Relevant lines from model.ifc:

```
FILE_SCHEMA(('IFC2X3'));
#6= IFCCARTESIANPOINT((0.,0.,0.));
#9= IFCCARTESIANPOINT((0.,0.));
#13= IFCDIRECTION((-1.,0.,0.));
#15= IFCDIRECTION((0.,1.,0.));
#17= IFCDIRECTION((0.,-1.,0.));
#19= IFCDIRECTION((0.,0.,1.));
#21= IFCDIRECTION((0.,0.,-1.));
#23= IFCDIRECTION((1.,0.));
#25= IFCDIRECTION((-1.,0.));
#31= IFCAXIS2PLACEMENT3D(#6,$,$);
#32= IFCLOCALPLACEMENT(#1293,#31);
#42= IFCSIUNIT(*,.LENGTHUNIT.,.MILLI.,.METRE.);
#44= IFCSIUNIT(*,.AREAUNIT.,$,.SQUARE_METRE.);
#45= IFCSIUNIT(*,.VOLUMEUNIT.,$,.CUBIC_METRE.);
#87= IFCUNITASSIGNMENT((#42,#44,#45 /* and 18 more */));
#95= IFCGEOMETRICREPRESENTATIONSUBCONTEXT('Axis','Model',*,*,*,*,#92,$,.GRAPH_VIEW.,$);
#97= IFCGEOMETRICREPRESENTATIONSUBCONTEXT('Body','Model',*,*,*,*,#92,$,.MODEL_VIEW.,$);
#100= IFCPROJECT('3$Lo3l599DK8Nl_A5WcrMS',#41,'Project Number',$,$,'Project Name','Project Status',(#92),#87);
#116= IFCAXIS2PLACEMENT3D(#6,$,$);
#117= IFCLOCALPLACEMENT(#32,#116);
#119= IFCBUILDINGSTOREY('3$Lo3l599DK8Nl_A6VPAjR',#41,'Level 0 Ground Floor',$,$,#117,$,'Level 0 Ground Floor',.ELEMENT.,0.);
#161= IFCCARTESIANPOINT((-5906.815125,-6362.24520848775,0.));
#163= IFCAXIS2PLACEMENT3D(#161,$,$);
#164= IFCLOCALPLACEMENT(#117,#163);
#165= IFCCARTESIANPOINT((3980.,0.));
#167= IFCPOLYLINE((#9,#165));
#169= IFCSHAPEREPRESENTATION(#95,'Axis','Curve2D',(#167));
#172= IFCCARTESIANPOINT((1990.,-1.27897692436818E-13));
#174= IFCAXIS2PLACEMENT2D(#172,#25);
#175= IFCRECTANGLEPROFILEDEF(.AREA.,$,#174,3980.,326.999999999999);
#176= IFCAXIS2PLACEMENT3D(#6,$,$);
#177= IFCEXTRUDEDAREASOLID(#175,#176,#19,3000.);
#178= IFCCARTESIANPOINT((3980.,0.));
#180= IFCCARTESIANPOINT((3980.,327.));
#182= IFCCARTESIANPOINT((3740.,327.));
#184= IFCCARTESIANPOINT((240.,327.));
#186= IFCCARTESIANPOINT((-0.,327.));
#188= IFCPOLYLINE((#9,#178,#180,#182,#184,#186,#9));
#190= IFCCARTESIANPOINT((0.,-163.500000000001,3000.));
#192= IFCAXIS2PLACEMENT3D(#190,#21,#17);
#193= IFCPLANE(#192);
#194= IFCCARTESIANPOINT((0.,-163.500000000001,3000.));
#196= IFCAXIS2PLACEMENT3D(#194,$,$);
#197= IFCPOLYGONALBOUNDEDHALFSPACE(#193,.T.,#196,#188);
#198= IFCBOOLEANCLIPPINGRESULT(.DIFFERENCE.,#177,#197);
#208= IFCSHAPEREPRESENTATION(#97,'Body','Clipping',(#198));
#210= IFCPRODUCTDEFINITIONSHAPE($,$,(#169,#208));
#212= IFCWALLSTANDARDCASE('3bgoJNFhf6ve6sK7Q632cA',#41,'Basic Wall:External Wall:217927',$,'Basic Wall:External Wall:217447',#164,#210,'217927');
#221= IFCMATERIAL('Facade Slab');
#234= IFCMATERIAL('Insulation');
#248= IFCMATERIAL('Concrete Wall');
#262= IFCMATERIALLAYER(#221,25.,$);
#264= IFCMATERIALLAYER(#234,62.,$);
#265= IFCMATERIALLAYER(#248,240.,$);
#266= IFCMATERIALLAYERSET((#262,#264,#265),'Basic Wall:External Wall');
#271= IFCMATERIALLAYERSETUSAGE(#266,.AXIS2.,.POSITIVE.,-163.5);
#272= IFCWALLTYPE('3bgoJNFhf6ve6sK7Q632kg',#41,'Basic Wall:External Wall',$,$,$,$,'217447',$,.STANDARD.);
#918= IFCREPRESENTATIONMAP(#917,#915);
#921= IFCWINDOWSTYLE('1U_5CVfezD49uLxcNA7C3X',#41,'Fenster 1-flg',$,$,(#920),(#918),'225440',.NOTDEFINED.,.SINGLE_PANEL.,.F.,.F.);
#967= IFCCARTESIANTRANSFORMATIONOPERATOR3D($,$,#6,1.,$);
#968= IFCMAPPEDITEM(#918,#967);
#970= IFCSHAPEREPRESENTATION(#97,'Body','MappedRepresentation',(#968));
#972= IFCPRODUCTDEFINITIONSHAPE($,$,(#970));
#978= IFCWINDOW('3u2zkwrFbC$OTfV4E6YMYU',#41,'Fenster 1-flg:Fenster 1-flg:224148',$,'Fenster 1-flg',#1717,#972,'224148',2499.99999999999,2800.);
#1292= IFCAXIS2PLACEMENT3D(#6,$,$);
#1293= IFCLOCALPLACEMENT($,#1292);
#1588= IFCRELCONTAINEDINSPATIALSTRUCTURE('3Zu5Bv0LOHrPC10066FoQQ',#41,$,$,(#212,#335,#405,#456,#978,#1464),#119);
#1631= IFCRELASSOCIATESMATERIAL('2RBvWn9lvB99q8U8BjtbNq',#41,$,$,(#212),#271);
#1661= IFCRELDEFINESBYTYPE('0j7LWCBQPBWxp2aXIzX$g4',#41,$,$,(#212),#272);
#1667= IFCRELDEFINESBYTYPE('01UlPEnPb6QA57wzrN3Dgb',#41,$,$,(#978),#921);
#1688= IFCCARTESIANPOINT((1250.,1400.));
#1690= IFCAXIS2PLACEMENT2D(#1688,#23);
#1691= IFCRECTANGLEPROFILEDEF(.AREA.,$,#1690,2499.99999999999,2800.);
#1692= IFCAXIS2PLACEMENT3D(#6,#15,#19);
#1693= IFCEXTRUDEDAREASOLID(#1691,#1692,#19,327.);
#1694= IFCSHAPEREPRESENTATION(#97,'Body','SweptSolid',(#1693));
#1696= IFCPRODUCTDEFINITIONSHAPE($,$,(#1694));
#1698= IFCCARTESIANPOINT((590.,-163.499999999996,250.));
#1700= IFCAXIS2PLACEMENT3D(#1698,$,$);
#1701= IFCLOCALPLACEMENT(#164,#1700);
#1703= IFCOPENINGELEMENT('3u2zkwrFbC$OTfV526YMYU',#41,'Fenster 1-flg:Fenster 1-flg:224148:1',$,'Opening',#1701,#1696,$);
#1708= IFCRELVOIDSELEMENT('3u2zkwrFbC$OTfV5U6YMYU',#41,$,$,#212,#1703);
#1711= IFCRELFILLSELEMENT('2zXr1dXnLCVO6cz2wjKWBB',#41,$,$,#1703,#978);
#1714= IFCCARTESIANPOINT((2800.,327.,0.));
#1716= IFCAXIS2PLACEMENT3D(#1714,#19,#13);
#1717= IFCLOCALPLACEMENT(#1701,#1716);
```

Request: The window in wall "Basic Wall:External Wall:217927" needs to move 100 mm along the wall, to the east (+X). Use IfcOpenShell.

```python
import ifcopenshell
import ifcopenshell.api.geometry
import ifcopenshell.util.placement
import ifcopenshell.util.unit

model = ifcopenshell.open("model.ifc")
unit_scale = ifcopenshell.util.unit.calculate_unit_scale(model)

window = model.by_guid("3u2zkwrFbC$OTfV4E6YMYU")
opening = window.FillsVoids[0].RelatingOpeningElement
wall = opening.VoidsElements[0].RelatingBuildingElement

wall_matrix = ifcopenshell.util.placement.get_local_placement(wall.ObjectPlacement)
shift = wall_matrix[:3, 0] * 0.1 / unit_scale
before = ifcopenshell.util.placement.get_local_placement(window.ObjectPlacement)[:3, 3].copy()

# The window is placed relative to its opening, so it follows when the opening moves.
matrix = ifcopenshell.util.placement.get_local_placement(opening.ObjectPlacement)
matrix[:3, 3] += shift
ifcopenshell.api.geometry.edit_object_placement(
    model, product=opening, matrix=matrix, is_si=False, should_transform_children=True
)

after = ifcopenshell.util.placement.get_local_placement(window.ObjectPlacement)[:3, 3]
print("window moved by", (after - before).round(3) + 0.0)

model.write("model_v2.ifc")
```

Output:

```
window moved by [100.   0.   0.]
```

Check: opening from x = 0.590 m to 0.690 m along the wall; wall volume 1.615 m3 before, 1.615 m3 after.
